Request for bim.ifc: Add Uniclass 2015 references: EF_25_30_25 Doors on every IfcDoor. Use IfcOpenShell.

First a look at what the model holds.

```python
import ifcopenshell

model = ifcopenshell.open("bim.ifc")
print(model.schema)
print("classifications:", [c.Name for c in model.by_type("IfcClassification")])
for ifc_class in ("IfcDoor", "IfcRoof", "IfcStair", "IfcWall", "IfcWindow"):
    print(ifc_class, len(model.by_type(ifc_class)))
```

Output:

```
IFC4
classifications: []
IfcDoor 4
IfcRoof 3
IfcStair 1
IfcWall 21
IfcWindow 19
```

```python
import ifcopenshell
import ifcopenshell.api.classification

model = ifcopenshell.open("bim.ifc")

system = ifcopenshell.api.classification.add_classification(model, classification="Uniclass 2015")

codes = {
    "IfcDoor": ("EF_25_30_25", "Doors"),
}
for ifc_class, (code, name) in codes.items():
    products = model.by_type(ifc_class)
    ifcopenshell.api.classification.add_reference(
        model, products=products, classification=system, identification=code, name=name
    )
    print(code, len(products))

model.write("bim_rev.ifc")
```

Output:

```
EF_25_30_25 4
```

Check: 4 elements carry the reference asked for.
